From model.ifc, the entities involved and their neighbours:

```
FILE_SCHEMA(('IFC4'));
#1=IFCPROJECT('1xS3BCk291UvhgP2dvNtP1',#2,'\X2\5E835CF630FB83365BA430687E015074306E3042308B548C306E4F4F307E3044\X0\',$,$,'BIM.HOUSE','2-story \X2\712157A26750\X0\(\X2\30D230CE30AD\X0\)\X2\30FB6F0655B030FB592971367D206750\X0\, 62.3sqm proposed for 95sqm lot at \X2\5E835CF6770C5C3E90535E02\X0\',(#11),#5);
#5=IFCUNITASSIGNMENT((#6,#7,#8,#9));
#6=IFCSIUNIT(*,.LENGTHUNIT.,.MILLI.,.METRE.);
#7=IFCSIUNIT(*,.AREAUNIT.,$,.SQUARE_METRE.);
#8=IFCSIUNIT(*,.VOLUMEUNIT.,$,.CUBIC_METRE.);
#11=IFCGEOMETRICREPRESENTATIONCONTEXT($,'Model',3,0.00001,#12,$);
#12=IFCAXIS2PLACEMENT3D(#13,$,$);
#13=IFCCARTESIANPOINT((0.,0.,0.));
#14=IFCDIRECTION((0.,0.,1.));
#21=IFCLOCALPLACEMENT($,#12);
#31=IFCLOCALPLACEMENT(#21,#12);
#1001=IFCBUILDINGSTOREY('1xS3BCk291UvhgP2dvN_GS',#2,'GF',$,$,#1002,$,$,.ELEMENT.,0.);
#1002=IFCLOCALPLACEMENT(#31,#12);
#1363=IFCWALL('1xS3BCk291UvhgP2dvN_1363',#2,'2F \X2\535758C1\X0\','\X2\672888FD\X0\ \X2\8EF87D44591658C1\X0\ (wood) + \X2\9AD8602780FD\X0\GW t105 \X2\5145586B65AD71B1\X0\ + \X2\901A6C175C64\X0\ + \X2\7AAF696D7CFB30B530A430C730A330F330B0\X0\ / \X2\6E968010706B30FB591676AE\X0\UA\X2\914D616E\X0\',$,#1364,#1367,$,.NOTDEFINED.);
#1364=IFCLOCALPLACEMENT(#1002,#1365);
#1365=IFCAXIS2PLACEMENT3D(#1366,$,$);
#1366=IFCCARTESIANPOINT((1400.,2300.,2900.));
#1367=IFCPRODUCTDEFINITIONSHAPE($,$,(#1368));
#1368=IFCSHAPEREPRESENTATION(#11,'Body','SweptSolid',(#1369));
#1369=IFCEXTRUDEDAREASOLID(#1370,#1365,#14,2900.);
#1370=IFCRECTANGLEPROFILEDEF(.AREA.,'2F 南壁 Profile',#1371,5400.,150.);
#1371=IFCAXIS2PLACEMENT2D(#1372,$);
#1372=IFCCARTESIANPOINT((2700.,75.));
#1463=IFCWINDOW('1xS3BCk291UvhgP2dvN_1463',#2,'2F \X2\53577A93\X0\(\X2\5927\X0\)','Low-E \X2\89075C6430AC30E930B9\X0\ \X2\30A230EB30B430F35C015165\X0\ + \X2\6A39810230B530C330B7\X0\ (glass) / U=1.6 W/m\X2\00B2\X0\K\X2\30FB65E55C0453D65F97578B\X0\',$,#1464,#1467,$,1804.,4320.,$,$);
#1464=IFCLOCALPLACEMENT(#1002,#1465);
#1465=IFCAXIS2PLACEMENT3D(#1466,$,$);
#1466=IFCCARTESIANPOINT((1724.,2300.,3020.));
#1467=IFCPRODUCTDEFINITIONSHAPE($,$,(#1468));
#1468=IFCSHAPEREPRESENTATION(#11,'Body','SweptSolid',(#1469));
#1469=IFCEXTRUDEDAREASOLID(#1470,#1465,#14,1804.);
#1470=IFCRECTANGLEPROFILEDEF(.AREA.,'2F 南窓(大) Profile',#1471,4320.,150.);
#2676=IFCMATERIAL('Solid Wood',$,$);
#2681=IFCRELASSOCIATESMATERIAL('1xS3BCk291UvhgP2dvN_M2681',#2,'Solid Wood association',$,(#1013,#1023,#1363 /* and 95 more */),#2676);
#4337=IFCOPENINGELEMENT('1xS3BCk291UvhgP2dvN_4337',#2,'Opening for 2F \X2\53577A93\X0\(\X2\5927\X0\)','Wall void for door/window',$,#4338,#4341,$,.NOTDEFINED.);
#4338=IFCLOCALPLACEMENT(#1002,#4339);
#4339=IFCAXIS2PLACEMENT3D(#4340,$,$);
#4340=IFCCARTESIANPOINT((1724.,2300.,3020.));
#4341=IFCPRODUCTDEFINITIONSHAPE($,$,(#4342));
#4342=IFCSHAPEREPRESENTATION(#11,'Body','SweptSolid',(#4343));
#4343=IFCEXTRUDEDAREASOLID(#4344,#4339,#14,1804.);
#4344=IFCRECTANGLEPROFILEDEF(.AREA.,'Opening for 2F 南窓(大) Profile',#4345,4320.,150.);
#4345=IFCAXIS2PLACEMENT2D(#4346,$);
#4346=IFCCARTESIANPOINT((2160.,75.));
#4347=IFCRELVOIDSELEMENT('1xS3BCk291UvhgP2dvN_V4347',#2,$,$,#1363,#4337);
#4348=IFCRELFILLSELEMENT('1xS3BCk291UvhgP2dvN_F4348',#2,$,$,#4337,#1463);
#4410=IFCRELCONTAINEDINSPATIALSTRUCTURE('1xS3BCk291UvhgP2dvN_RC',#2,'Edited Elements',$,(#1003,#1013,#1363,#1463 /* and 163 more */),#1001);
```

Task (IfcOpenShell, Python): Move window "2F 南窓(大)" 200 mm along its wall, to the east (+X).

```python
import ifcopenshell
import ifcopenshell.api.geometry
import ifcopenshell.util.placement

model = ifcopenshell.open("model.ifc")

window = model.by_guid("1xS3BCk291UvhgP2dvN_1463")
opening = window.FillsVoids[0].RelatingOpeningElement
wall = opening.VoidsElements[0].RelatingBuildingElement

wall_matrix = ifcopenshell.util.placement.get_local_placement(wall.ObjectPlacement)
shift = wall_matrix[:3, 0] * 200.0
before = ifcopenshell.util.placement.get_local_placement(window.ObjectPlacement)[:3, 3].copy()

# The window is not placed relative to its opening, so move both.
for product in (opening, window):
    matrix = ifcopenshell.util.placement.get_local_placement(product.ObjectPlacement)
    matrix[:3, 3] += shift
    ifcopenshell.api.geometry.edit_object_placement(model, product=product, matrix=matrix, is_si=False)

after = ifcopenshell.util.placement.get_local_placement(window.ObjectPlacement)[:3, 3]
print("window moved by", (after - before).round(3) + 0.0)

model.write("model_edited.ifc")
```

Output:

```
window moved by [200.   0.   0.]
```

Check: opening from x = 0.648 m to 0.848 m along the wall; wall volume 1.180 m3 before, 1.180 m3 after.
